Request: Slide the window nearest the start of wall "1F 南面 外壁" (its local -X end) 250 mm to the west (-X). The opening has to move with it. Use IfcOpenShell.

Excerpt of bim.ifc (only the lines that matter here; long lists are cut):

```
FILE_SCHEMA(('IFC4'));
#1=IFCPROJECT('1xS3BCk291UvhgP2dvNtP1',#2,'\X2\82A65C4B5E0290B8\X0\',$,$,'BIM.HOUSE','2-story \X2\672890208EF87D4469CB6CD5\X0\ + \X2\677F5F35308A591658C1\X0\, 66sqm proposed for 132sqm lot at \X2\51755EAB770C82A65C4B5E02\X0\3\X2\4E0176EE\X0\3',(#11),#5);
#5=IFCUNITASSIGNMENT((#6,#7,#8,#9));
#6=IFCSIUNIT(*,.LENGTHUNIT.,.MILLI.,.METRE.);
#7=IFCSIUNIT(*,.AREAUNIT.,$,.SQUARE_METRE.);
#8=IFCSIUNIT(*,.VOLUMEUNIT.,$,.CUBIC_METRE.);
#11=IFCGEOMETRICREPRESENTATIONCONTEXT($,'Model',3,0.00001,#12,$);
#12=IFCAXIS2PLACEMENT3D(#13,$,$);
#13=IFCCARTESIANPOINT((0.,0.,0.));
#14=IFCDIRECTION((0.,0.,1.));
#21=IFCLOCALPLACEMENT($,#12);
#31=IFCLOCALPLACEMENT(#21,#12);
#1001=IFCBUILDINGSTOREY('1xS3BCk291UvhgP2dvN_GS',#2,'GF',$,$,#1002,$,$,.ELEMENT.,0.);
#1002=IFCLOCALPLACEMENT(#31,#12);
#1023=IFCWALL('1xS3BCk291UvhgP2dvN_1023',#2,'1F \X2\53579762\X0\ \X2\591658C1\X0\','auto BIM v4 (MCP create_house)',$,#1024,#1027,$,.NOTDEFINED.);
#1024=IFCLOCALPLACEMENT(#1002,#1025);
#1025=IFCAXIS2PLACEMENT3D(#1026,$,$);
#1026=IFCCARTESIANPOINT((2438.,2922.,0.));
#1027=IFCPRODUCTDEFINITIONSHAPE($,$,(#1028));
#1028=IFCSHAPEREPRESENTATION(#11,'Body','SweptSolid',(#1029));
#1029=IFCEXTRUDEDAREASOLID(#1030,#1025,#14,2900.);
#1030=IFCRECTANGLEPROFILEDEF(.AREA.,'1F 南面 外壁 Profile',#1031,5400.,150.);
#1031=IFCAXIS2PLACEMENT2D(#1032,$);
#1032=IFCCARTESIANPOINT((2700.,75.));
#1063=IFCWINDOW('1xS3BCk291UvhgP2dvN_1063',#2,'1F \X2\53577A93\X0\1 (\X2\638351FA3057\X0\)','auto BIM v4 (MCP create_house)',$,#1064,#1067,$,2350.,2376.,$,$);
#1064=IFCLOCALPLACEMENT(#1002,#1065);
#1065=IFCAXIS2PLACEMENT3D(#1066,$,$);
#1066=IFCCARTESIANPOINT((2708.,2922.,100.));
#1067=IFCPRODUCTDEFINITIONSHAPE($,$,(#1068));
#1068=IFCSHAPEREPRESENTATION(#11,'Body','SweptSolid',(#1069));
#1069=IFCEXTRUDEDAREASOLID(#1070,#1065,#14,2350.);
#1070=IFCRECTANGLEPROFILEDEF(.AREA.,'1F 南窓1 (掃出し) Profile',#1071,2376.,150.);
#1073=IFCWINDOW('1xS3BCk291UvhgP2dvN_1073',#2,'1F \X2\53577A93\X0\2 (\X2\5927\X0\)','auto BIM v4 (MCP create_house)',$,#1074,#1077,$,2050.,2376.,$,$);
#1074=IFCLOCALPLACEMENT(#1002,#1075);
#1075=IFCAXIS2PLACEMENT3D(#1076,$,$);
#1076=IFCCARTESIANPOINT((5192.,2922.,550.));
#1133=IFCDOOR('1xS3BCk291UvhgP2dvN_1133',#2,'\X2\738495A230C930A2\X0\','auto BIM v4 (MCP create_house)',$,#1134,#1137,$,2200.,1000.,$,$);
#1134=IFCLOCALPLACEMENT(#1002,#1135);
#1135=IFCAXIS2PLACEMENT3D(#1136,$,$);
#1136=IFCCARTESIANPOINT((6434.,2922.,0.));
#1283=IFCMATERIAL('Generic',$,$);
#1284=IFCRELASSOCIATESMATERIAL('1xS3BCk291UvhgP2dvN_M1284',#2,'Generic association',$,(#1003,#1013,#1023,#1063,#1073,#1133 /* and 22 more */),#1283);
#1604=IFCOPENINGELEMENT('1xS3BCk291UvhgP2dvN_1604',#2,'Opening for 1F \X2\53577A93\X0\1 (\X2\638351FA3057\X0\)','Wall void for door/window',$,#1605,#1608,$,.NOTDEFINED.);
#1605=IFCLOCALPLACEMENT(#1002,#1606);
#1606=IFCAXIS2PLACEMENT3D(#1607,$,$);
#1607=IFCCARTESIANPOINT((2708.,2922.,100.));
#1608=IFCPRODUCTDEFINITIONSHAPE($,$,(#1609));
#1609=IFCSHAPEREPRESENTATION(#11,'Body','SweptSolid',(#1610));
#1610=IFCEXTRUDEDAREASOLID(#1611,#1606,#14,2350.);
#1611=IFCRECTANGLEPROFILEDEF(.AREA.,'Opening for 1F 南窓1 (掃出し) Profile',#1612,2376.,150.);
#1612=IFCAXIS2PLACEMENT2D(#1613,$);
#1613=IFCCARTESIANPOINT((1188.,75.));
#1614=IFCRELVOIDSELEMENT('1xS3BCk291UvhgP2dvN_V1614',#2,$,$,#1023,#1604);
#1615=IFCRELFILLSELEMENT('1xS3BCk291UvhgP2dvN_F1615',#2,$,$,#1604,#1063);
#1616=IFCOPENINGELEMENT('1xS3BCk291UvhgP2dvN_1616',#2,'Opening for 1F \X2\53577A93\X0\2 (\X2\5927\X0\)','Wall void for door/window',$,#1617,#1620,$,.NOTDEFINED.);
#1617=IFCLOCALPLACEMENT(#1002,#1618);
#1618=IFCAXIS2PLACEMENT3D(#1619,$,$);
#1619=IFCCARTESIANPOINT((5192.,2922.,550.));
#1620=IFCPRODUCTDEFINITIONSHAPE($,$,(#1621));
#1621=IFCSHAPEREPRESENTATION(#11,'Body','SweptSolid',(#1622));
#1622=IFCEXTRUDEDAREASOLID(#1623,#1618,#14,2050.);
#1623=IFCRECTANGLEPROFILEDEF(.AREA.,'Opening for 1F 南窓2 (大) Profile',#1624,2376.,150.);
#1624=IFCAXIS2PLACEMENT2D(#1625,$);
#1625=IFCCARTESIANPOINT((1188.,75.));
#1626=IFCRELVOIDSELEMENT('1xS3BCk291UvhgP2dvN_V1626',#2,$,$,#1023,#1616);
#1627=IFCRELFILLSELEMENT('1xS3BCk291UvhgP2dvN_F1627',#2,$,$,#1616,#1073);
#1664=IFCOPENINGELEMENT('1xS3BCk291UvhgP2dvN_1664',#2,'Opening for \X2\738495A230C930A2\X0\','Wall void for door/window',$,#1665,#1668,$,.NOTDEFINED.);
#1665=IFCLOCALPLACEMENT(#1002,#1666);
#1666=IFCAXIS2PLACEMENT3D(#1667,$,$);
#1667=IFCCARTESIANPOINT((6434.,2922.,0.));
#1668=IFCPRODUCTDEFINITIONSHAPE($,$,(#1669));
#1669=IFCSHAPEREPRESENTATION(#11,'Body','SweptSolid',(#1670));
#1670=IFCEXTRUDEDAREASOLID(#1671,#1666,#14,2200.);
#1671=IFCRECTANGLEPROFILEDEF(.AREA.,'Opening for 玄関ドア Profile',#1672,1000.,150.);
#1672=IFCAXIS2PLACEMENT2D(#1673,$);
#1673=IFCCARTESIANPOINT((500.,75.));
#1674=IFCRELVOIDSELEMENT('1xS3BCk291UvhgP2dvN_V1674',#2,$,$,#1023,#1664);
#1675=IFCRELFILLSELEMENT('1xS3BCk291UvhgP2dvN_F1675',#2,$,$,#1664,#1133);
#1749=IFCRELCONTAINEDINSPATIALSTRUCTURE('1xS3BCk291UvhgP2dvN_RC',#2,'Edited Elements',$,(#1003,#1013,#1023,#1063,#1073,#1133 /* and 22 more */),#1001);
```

```python
import ifcopenshell
import ifcopenshell.api.geometry
import ifcopenshell.util.placement
import ifcopenshell.util.unit

model = ifcopenshell.open("bim.ifc")
unit_scale = ifcopenshell.util.unit.calculate_unit_scale(model)

window = model.by_guid("1xS3BCk291UvhgP2dvN_1063")
opening = window.FillsVoids[0].RelatingOpeningElement
wall = opening.VoidsElements[0].RelatingBuildingElement

wall_matrix = ifcopenshell.util.placement.get_local_placement(wall.ObjectPlacement)
shift = wall_matrix[:3, 0] * -0.25 / unit_scale
before = ifcopenshell.util.placement.get_local_placement(window.ObjectPlacement)[:3, 3].copy()

# The window is not placed relative to its opening, so move both.
for product in (opening, window):
    matrix = ifcopenshell.util.placement.get_local_placement(product.ObjectPlacement)
    matrix[:3, 3] += shift
    ifcopenshell.api.geometry.edit_object_placement(model, product=product, matrix=matrix, is_si=False)

after = ifcopenshell.util.placement.get_local_placement(window.ObjectPlacement)[:3, 3]
print("window moved by", (after - before).round(3) + 0.0)

model.write("bim_updated.ifc")
```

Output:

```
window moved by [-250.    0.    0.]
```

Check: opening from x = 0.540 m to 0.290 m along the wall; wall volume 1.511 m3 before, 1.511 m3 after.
